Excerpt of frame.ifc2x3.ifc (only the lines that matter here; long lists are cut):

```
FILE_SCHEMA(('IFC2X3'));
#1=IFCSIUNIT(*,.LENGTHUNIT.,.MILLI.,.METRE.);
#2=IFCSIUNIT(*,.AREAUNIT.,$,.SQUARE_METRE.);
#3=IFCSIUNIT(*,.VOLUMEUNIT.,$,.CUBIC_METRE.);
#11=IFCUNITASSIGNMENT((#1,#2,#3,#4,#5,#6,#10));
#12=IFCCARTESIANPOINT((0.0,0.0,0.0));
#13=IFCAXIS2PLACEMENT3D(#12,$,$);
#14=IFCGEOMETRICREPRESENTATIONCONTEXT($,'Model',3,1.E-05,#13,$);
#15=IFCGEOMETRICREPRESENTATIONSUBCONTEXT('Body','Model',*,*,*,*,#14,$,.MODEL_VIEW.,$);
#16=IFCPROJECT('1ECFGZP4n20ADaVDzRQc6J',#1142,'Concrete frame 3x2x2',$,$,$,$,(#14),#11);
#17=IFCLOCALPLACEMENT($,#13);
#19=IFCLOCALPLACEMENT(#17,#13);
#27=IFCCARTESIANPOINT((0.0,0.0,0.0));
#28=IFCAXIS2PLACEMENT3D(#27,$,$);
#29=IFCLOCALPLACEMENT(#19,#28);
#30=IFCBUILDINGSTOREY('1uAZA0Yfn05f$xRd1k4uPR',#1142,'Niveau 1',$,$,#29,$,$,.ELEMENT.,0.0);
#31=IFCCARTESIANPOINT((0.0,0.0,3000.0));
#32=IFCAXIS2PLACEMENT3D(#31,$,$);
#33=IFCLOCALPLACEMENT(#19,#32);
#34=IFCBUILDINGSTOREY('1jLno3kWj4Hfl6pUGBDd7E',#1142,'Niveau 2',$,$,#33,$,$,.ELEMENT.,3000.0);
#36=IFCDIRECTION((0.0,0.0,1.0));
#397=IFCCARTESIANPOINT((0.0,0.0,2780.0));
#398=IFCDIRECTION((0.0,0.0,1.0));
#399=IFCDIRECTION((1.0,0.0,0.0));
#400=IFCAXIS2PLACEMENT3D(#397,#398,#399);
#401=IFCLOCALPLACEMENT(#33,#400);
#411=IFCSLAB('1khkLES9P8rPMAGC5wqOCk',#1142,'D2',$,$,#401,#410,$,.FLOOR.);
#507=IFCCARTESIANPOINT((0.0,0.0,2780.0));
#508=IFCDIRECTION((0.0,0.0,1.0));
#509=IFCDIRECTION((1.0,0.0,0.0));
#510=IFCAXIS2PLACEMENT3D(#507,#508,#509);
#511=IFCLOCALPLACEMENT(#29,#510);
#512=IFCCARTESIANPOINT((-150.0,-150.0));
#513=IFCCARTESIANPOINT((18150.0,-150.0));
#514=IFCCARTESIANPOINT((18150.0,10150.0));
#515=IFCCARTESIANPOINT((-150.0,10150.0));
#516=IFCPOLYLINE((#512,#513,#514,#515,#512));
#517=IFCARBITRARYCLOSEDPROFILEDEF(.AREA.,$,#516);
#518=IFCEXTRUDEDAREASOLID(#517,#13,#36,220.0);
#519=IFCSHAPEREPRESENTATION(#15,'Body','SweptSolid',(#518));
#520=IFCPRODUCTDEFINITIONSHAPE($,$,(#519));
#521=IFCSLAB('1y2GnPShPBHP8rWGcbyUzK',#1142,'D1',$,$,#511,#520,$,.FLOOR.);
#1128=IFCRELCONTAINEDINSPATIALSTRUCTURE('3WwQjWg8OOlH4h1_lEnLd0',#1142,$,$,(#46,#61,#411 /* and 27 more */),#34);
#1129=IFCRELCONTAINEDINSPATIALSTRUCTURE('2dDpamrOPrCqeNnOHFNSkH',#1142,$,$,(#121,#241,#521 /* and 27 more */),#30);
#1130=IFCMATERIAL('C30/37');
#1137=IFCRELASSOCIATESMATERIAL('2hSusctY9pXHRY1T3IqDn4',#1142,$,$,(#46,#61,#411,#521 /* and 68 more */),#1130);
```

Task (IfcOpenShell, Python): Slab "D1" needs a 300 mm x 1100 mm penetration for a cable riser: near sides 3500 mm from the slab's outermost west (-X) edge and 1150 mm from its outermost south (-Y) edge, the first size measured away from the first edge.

```python
import numpy as np
import ifcopenshell
import ifcopenshell.api.feature
import ifcopenshell.api.geometry
import ifcopenshell.api.root
import ifcopenshell.geom
import ifcopenshell.util.placement
import ifcopenshell.util.representation
import ifcopenshell.util.shape
import ifcopenshell.util.unit

model = ifcopenshell.open("frame.ifc2x3.ifc")
unit_scale = ifcopenshell.util.unit.calculate_unit_scale(model)
settings = ifcopenshell.geom.settings()


def volume(element):
    """Net volume in cubic metres, openings subtracted."""
    shape = ifcopenshell.geom.create_shape(settings, element)
    return ifcopenshell.util.shape.get_volume(shape.geometry)


slab = model.by_id(521)
before = volume(slab)

# Extent in the slab's own axes, in metres. The edges named are its -X and -Y sides.
slab_shape = ifcopenshell.geom.create_shape(settings, slab)
vertices = ifcopenshell.util.shape.get_vertices(slab_shape.geometry)
x_min, y_min, bottom = vertices.min(axis=0)
top = vertices[:, 2].max()

opening = ifcopenshell.api.root.create_entity(model, ifc_class="IfcOpeningElement", name="Cable riser opening")
context = ifcopenshell.util.representation.get_context(model, "Model", "Body", "MODEL_VIEW")
width, depth = 0.3, 1.1
outline = [(0.0, 0.0), (width, 0.0), (width, depth), (0.0, depth), (0.0, 0.0)]
# Overshoot both faces by 50 mm so the cut is clean.
shape = ifcopenshell.api.geometry.add_slab_representation(
    model, context=context, depth=top - bottom + 0.1, polyline=outline
)
ifcopenshell.api.geometry.assign_representation(model, product=opening, representation=shape)

matrix = ifcopenshell.util.placement.get_local_placement(slab.ObjectPlacement)
matrix[:, 3] = matrix @ np.append(np.array([x_min + 3.5, y_min + 1.15, bottom - 0.05]) / unit_scale, 1.0)
ifcopenshell.api.geometry.edit_object_placement(model, product=opening, matrix=matrix, is_si=False)
ifcopenshell.api.feature.add_feature(model, feature=opening, element=slab)

after = volume(slab)

print(f"slab volume {before:.3f} -> {after:.3f} m3")

model.write("frame.ifc2x3_v2.ifc")
```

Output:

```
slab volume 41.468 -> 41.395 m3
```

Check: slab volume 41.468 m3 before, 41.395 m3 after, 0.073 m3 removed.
